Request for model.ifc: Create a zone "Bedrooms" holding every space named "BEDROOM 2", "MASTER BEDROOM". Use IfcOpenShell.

First a look at what the model holds.

```python
import ifcopenshell

model = ifcopenshell.open("model.ifc")
print(model.schema)
seen = {}
for space in model.by_type("IfcSpace"):
    seen[space.LongName] = seen.get(space.LongName, 0) + 1
for name, count in sorted(seen.items(), key=str):
    print(count, "x", name)
print("zones:", [z.Name for z in model.by_type("IfcZone")][:20])
```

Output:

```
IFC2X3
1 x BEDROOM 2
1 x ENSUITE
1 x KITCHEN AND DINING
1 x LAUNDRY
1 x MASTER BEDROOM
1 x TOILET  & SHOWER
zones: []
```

```python
import ifcopenshell
import ifcopenshell.api.group
import ifcopenshell.api.root

model = ifcopenshell.open("model.ifc")

names = {"BEDROOM 2", "MASTER BEDROOM"}
spaces = [s for s in model.by_type("IfcSpace") if s.LongName in names]

zone = ifcopenshell.api.root.create_entity(model, ifc_class="IfcZone", name="Bedrooms")
ifcopenshell.api.group.assign_group(model, products=spaces, group=zone)
print(len(spaces), "spaces in", zone.Name)

model.write("model_edited.ifc")
```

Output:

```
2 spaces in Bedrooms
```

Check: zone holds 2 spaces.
